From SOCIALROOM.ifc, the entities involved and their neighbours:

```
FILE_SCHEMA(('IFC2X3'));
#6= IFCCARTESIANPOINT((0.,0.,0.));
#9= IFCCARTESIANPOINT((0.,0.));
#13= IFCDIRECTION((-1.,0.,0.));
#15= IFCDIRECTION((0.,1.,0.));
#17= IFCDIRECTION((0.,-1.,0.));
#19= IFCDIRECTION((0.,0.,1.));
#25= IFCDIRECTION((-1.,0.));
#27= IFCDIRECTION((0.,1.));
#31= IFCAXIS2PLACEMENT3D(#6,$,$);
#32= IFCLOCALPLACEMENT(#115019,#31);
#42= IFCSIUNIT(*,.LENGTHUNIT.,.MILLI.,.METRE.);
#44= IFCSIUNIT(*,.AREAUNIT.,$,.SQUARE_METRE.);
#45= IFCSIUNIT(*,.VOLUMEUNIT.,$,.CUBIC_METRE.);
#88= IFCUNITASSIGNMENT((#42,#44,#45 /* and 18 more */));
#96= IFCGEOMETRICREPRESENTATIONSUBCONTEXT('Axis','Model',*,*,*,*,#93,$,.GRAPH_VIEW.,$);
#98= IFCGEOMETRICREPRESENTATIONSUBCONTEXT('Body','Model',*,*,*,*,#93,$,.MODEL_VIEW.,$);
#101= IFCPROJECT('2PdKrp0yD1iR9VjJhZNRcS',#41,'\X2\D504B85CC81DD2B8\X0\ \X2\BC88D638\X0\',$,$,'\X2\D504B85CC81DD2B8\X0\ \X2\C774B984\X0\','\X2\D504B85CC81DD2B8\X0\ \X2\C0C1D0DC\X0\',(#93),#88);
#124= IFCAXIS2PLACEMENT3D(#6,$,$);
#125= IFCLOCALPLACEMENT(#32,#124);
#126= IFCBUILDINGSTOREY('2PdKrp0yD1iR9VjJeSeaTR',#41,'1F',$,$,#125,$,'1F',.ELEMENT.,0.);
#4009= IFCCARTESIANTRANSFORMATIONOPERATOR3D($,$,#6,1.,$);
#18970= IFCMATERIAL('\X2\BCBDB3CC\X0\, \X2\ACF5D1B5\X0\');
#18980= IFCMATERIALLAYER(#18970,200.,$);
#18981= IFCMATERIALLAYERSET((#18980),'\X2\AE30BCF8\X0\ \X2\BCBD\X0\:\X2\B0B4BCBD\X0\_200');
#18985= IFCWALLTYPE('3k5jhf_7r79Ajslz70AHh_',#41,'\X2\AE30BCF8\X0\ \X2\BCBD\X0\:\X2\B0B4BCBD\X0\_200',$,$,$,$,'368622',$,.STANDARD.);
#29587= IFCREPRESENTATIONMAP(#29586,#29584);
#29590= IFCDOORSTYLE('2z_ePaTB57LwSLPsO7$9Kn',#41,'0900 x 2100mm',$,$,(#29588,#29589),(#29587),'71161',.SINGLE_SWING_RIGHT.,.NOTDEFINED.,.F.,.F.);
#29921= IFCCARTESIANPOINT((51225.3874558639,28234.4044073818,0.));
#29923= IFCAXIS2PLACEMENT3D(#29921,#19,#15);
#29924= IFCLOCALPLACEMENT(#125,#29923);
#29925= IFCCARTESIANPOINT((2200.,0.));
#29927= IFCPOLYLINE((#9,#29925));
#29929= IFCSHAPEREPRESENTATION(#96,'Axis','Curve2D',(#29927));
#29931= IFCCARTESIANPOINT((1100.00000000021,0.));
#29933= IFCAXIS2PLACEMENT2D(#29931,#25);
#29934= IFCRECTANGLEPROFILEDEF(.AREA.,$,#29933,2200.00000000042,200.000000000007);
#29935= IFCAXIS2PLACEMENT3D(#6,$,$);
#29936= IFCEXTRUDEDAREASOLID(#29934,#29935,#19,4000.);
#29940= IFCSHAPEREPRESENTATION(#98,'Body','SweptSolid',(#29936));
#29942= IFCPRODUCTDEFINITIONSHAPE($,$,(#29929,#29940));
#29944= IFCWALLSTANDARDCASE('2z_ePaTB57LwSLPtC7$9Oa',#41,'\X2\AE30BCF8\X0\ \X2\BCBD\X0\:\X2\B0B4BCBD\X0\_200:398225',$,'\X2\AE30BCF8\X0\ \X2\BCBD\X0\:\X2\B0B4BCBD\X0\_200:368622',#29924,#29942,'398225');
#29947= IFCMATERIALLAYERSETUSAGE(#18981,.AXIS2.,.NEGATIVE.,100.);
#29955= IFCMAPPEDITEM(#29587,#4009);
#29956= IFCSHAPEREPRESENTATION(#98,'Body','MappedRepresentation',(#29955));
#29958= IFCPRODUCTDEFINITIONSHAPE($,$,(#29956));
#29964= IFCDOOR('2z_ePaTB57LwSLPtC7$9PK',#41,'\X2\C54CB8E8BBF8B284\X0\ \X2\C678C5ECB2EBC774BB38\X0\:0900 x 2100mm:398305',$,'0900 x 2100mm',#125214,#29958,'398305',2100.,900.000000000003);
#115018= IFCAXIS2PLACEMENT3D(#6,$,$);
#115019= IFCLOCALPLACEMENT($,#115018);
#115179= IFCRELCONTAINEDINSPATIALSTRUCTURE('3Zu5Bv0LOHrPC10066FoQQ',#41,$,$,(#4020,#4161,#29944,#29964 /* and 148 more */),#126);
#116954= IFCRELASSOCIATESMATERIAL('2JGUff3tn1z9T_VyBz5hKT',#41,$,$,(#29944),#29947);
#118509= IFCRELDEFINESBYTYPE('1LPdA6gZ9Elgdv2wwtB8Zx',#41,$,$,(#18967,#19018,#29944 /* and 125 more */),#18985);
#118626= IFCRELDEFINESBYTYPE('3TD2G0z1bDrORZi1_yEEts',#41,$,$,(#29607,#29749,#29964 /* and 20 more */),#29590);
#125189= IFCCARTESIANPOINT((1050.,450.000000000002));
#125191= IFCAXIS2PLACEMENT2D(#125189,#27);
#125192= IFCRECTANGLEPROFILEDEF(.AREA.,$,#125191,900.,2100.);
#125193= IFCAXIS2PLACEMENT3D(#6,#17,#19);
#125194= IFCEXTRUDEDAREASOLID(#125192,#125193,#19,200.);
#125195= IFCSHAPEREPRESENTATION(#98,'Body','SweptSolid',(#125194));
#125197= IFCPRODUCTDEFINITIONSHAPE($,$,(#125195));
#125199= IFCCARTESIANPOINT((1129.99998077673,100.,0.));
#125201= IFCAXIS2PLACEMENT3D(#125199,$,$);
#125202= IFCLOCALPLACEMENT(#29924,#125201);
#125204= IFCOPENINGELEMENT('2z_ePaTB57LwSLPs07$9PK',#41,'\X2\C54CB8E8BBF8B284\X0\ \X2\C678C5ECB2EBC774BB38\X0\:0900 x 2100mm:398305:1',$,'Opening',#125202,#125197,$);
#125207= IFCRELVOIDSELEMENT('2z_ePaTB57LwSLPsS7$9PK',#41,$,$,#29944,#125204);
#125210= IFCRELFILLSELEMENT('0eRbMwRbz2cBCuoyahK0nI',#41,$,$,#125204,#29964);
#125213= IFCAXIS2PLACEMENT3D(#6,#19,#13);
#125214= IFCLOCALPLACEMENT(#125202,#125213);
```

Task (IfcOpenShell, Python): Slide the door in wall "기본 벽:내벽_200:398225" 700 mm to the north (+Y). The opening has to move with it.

```python
import ifcopenshell
import ifcopenshell.api.geometry
import ifcopenshell.util.placement

model = ifcopenshell.open("SOCIALROOM.ifc")

door = model.by_guid("2z_ePaTB57LwSLPtC7$9PK")
opening = door.FillsVoids[0].RelatingOpeningElement
wall = opening.VoidsElements[0].RelatingBuildingElement

wall_matrix = ifcopenshell.util.placement.get_local_placement(wall.ObjectPlacement)
shift = wall_matrix[:3, 0] * 700.0
before = ifcopenshell.util.placement.get_local_placement(door.ObjectPlacement)[:3, 3].copy()

# The door is placed relative to its opening, so it follows when the opening moves.
matrix = ifcopenshell.util.placement.get_local_placement(opening.ObjectPlacement)
matrix[:3, 3] += shift
ifcopenshell.api.geometry.edit_object_placement(
    model, product=opening, matrix=matrix, is_si=False, should_transform_children=True
)

after = ifcopenshell.util.placement.get_local_placement(door.ObjectPlacement)[:3, 3]
print("door moved by", (after - before).round(3) + 0.0)

model.write("SOCIALROOM-out.ifc")
```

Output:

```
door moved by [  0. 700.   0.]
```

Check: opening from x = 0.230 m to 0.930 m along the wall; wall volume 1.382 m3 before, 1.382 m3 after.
